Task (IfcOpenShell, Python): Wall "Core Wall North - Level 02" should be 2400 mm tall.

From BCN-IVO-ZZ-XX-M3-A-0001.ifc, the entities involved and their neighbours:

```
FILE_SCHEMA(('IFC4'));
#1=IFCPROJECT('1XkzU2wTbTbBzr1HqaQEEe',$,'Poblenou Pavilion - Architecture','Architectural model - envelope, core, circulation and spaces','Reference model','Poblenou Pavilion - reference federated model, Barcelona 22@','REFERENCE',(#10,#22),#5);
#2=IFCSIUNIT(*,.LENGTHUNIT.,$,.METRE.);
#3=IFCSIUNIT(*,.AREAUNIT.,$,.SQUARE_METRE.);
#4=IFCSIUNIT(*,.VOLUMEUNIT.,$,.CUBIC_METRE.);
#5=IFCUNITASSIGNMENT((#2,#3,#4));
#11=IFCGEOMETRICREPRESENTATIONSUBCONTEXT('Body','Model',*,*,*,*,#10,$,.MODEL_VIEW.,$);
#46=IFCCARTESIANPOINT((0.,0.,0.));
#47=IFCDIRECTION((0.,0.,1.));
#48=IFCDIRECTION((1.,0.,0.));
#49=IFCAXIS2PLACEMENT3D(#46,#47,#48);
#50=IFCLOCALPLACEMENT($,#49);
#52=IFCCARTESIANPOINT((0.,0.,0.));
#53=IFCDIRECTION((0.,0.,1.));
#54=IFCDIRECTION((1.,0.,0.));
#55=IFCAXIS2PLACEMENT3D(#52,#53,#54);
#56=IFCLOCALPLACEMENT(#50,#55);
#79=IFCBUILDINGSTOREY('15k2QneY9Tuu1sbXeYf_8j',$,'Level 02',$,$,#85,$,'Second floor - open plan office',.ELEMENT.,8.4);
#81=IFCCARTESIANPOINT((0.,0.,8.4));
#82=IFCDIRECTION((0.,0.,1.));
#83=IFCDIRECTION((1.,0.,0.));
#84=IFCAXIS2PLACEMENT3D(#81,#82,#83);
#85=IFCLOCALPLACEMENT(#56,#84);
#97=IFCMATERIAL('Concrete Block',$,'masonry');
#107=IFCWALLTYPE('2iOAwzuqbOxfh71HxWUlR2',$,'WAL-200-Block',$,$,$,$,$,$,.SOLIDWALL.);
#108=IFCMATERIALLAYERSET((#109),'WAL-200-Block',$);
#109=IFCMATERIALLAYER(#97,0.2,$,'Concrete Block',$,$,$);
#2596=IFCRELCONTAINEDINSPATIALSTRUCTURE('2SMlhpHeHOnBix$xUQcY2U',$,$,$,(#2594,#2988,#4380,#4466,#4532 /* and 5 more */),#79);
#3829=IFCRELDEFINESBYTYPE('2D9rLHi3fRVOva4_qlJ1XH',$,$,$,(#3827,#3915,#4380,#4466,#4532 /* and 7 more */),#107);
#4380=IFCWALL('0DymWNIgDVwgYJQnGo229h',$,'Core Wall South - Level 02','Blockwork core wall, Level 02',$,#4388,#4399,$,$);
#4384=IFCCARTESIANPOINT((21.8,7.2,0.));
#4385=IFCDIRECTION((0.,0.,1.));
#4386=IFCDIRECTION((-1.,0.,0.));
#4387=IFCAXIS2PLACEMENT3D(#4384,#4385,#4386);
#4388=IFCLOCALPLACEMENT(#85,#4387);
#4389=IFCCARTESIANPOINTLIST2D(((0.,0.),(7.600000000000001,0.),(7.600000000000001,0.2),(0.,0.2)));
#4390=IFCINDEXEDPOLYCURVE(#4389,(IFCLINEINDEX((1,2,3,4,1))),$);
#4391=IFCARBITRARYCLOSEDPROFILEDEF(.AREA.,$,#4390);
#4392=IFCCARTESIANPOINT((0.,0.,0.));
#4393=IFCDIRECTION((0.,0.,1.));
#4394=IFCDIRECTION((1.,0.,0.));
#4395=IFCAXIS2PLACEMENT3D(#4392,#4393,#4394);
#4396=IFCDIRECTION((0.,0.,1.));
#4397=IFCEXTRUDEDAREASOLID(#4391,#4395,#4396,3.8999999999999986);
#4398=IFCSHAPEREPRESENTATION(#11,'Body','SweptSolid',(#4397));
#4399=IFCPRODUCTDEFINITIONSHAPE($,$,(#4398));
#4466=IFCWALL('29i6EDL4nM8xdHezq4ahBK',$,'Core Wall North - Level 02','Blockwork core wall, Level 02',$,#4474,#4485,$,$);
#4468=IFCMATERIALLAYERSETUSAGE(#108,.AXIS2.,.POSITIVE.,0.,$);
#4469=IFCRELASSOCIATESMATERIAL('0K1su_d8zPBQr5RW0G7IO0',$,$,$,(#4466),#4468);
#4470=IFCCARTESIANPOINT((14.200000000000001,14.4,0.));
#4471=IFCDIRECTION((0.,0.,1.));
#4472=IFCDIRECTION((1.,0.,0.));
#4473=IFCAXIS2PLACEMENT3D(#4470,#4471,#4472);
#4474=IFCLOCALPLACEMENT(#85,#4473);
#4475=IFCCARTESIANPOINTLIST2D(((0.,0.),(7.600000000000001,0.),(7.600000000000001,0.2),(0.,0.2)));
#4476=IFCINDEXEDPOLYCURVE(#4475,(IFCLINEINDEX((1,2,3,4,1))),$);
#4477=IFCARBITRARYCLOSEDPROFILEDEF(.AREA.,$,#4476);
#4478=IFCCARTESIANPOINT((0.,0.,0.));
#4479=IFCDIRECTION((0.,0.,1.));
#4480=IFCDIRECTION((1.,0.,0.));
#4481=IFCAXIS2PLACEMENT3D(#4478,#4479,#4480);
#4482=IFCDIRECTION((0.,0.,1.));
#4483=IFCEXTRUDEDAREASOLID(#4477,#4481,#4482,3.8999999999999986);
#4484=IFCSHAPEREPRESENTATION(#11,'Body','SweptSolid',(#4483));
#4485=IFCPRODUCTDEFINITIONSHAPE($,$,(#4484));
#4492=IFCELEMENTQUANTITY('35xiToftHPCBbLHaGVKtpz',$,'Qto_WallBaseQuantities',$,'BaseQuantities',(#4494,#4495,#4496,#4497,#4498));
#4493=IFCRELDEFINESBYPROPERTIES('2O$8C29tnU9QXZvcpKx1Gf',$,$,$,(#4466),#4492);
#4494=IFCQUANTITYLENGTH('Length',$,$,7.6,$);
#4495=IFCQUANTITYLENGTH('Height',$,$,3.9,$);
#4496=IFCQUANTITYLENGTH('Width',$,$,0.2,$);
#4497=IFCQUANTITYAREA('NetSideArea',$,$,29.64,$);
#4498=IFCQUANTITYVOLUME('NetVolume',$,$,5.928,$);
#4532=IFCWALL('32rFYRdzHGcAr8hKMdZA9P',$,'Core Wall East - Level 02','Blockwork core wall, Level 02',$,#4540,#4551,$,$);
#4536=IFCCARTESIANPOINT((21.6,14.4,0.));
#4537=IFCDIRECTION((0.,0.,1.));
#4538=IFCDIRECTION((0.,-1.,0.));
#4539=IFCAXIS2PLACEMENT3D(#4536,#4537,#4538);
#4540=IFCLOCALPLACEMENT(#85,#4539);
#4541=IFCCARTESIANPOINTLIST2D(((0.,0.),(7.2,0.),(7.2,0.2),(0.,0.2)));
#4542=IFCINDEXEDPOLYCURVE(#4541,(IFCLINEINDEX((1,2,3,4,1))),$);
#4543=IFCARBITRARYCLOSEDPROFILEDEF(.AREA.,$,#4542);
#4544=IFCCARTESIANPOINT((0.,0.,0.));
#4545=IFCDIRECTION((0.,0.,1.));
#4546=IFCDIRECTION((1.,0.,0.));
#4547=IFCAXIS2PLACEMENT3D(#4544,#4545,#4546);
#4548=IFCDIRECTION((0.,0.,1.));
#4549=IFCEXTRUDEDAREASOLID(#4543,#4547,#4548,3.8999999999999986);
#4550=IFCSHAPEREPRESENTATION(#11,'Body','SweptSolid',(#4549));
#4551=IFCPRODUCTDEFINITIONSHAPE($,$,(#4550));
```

```python
import ifcopenshell
import ifcopenshell.api.pset
import ifcopenshell.geom
import ifcopenshell.util.element
import ifcopenshell.util.representation
import ifcopenshell.util.shape
import ifcopenshell.util.unit

model = ifcopenshell.open("BCN-IVO-ZZ-XX-M3-A-0001.ifc")
area_scale = ifcopenshell.util.unit.calculate_unit_scale(model, "AREAUNIT")
volume_scale = ifcopenshell.util.unit.calculate_unit_scale(model, "VOLUMEUNIT")
settings = ifcopenshell.geom.settings()


def volume(element):
    """Net volume in cubic metres, openings subtracted."""
    shape = ifcopenshell.geom.create_shape(settings, element)
    return ifcopenshell.util.shape.get_volume(shape.geometry)


wall = model.by_guid("29i6EDL4nM8xdHezq4ahBK")
before = volume(wall)

body = ifcopenshell.util.representation.get_representation(wall, "Model", "Body")
solid = body.Items[0]
old_height = solid.Depth
solid.Depth = 2.4
after = volume(wall)
thickness = 0.2  # wall thickness in metres

# Update the stored height, areas and volumes.
qto = model.by_id(ifcopenshell.util.element.get_pset(wall, "Qto_WallBaseQuantities", should_inherit=False)["id"])
ifcopenshell.api.pset.edit_qto(model, qto=qto, properties={
    "Height": solid.Depth,
    "NetSideArea": after / thickness / area_scale,
    "NetVolume": after / volume_scale,
})

print(f"height {old_height:g} -> {solid.Depth:g}, volume {before:.3f} -> {after:.3f} m3")

model.write("BCN-IVO-ZZ-XX-M3-A-0001_edited.ifc")
```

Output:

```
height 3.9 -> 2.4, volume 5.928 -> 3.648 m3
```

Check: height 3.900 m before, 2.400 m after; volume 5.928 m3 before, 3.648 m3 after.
